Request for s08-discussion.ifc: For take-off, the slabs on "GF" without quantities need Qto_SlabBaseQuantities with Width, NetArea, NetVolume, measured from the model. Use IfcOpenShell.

First a look at what the model holds.

```python
import ifcopenshell
import ifcopenshell.util.element
import ifcopenshell.util.unit

model = ifcopenshell.open("s08-discussion.ifc")
print(model.schema)
for unit_type in ("LENGTHUNIT", "AREAUNIT", "VOLUMEUNIT"):
    print(unit_type, ifcopenshell.util.unit.calculate_unit_scale(model, unit_type))
storey = next(s for s in model.by_type("IfcBuildingStorey") if s.Name == "GF")
slabs = [e for e in ifcopenshell.util.element.get_decomposition(storey) if e.is_a("IfcSlab")]
for e in sorted(slabs, key=lambda e: e.id()):
    print(e.id(), e.is_a(), e.Name, list(ifcopenshell.util.element.get_psets(e, qtos_only=True)), sep=" | ")
```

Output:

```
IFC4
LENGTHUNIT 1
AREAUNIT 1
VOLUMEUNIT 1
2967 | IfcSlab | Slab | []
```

```python
import ifcopenshell
import ifcopenshell.api.pset
import ifcopenshell.geom
import ifcopenshell.util.element
import ifcopenshell.util.shape
import ifcopenshell.util.unit

model = ifcopenshell.open("s08-discussion.ifc")
unit_scale = ifcopenshell.util.unit.calculate_unit_scale(model)
area_scale = ifcopenshell.util.unit.calculate_unit_scale(model, "AREAUNIT")
volume_scale = ifcopenshell.util.unit.calculate_unit_scale(model, "VOLUMEUNIT")
settings = ifcopenshell.geom.settings()

storey = next(s for s in model.by_type("IfcBuildingStorey") if s.Name == "GF")
slabs = [e for e in ifcopenshell.util.element.get_decomposition(storey) if e.is_a("IfcSlab")]

for e in sorted(slabs, key=lambda e: e.id()):
    if ifcopenshell.util.element.get_psets(e, qtos_only=True, should_inherit=False):
        continue
    # Geometry comes back in metres, in the element's own axes.
    shape = ifcopenshell.geom.create_shape(settings, e)
    values = {
        "Width": ifcopenshell.util.shape.get_z(shape.geometry) / unit_scale,
        "NetArea": ifcopenshell.util.shape.get_footprint_area(shape.geometry) / area_scale,
        "NetVolume": ifcopenshell.util.shape.get_volume(shape.geometry) / volume_scale,
    }
    qto = ifcopenshell.api.pset.add_qto(model, product=e, name="Qto_SlabBaseQuantities")
    ifcopenshell.api.pset.edit_qto(model, qto=qto, properties=values)
    print(e.id(), {k: round(v, 3) for k, v in values.items()})

model.write("s08-discussion_updated.ifc")
```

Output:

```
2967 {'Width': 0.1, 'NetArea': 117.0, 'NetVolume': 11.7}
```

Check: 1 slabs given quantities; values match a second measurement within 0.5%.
